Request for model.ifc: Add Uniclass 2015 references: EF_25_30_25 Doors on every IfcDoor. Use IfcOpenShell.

First a look at what the model holds.

```python
import ifcopenshell

model = ifcopenshell.open("model.ifc")
print(model.schema)
print("classifications:", [c.Name for c in model.by_type("IfcClassification")])
for ifc_class in ("IfcDoor", "IfcRoof", "IfcStair", "IfcWall", "IfcWindow"):
    print(ifc_class, len(model.by_type(ifc_class)))
```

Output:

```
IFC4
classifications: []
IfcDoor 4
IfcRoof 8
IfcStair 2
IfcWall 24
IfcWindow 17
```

```python
import ifcopenshell
import ifcopenshell.api.classification

model = ifcopenshell.open("model.ifc")

system = ifcopenshell.api.classification.add_classification(model, classification="Uniclass 2015")

codes = {
    "IfcDoor": ("EF_25_30_25", "Doors"),
}
for ifc_class, (code, name) in codes.items():
    products = model.by_type(ifc_class)
    ifcopenshell.api.classification.add_reference(
        model, products=products, classification=system, identification=code, name=name
    )
    print(code, len(products))

model.write("model_updated.ifc")
```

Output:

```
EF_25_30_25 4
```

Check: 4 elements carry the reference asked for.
